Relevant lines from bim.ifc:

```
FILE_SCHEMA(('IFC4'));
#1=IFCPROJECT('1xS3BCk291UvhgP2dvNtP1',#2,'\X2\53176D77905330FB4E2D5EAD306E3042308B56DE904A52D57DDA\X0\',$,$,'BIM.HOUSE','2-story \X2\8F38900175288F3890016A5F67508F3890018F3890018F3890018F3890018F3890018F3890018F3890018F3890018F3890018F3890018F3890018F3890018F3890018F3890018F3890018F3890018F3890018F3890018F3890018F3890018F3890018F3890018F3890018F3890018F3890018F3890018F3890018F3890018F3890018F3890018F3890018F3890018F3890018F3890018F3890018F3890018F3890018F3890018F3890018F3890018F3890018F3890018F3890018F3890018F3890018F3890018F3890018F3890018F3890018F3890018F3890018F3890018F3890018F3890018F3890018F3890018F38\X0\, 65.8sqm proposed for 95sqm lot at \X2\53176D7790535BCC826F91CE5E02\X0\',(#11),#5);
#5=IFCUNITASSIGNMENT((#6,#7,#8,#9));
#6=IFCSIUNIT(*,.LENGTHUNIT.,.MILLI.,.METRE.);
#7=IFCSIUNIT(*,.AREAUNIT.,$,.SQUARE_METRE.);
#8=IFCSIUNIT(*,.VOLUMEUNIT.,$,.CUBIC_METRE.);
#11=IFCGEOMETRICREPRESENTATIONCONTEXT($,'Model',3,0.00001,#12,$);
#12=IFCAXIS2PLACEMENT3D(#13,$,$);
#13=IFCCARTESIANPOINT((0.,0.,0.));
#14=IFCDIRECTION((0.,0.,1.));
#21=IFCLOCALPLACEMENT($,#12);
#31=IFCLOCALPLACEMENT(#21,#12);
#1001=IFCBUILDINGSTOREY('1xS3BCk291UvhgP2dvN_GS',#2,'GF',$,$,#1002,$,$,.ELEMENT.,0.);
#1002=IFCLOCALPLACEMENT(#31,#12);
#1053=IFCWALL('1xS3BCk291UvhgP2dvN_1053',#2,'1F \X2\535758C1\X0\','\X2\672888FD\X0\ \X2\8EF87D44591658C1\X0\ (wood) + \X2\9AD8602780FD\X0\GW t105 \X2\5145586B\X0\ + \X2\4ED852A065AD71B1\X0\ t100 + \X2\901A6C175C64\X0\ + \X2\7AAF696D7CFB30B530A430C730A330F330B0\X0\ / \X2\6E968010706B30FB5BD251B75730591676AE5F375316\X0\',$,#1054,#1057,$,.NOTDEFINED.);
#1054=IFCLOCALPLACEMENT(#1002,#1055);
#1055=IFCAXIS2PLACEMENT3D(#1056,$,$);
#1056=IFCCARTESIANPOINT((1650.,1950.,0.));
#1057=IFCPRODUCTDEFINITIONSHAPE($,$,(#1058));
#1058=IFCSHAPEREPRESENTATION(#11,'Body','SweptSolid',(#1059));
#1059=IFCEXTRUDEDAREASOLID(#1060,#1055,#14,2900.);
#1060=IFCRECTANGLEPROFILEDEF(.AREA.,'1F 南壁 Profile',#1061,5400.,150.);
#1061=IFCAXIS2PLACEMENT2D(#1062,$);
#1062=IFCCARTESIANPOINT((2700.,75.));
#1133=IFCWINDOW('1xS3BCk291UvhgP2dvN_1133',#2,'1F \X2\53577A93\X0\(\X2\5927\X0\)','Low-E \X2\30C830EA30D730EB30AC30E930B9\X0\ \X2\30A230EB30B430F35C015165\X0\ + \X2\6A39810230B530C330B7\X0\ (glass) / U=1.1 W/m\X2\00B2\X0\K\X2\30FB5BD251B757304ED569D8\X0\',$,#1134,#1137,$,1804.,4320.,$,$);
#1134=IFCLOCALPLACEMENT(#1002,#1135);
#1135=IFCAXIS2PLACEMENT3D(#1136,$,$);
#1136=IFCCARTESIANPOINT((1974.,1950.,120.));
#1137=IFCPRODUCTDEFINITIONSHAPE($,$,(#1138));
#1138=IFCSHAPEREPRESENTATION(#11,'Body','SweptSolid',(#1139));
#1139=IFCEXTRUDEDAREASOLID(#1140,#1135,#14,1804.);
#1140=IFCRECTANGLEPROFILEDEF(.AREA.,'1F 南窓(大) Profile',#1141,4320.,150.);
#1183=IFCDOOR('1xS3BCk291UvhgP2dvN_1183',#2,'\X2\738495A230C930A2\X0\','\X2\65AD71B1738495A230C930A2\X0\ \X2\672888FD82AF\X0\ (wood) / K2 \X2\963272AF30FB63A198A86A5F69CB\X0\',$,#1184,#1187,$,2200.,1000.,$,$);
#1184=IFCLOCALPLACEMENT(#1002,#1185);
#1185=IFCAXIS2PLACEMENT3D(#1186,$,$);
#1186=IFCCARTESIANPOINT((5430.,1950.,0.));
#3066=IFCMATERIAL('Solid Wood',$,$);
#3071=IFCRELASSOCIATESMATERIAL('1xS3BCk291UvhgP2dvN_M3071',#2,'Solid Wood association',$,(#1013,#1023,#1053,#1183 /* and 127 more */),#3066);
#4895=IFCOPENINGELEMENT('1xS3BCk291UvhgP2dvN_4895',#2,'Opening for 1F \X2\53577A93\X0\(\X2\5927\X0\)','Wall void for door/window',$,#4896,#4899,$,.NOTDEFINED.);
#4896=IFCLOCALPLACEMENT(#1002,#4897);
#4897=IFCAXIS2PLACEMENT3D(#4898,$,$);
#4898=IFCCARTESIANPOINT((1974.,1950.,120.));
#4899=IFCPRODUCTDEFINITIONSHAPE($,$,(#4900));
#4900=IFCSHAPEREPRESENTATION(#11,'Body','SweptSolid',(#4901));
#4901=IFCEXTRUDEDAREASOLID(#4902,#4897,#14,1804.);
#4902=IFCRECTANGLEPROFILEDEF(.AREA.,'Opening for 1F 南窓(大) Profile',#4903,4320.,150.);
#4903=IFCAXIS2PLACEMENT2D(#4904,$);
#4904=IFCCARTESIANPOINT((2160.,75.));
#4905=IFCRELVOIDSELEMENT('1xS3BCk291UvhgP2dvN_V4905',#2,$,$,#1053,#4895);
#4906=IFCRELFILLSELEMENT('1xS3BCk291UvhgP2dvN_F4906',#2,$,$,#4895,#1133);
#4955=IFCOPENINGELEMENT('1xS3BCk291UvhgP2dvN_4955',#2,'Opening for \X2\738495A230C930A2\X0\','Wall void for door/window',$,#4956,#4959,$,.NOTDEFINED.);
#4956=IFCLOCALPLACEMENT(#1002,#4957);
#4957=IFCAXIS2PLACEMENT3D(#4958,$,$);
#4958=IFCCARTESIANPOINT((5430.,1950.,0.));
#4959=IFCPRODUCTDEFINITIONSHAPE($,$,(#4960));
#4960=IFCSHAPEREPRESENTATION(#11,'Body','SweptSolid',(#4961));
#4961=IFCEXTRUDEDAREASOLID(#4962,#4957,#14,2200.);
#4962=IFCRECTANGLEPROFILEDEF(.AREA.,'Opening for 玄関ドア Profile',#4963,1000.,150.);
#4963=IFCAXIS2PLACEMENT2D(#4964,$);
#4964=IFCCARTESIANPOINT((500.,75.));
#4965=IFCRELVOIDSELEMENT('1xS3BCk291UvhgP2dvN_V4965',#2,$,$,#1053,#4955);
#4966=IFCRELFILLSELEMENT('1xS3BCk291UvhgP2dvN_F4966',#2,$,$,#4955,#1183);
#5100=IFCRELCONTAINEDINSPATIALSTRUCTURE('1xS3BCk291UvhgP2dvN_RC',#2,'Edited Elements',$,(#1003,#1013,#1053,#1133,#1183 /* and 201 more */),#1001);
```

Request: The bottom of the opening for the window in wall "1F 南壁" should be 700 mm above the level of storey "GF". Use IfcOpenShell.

```python
import numpy as np
import ifcopenshell
import ifcopenshell.api.geometry
import ifcopenshell.geom
import ifcopenshell.util.element
import ifcopenshell.util.placement
import ifcopenshell.util.shape
import ifcopenshell.util.unit

model = ifcopenshell.open("bim.ifc")
unit_scale = ifcopenshell.util.unit.calculate_unit_scale(model)

window = model.by_guid("1xS3BCk291UvhgP2dvN_1133")
opening = window.FillsVoids[0].RelatingOpeningElement
storey = ifcopenshell.util.element.get_container(window, ifc_class="IfcBuildingStorey")
level = ifcopenshell.util.placement.get_local_placement(storey.ObjectPlacement)[2, 3]

# The opening's origin need not be at the sill, so measure its lowest point.
shape = ifcopenshell.geom.create_shape(ifcopenshell.geom.settings(), opening)
bottom = ifcopenshell.util.shape.get_shape_bottom_elevation(shape, shape.geometry) / unit_scale
dz = level + 700.0 - bottom

shift = np.array([0.0, 0.0, dz])
# The window is not placed relative to its opening, so move both.
for product in (opening, window):
    matrix = ifcopenshell.util.placement.get_local_placement(product.ObjectPlacement)
    matrix[:3, 3] += shift
    ifcopenshell.api.geometry.edit_object_placement(model, product=product, matrix=matrix, is_si=False)

print(f"moved by {dz * unit_scale:+.3f} m")

model.write("bim_rev.ifc")
```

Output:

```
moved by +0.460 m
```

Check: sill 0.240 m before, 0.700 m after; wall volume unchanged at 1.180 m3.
